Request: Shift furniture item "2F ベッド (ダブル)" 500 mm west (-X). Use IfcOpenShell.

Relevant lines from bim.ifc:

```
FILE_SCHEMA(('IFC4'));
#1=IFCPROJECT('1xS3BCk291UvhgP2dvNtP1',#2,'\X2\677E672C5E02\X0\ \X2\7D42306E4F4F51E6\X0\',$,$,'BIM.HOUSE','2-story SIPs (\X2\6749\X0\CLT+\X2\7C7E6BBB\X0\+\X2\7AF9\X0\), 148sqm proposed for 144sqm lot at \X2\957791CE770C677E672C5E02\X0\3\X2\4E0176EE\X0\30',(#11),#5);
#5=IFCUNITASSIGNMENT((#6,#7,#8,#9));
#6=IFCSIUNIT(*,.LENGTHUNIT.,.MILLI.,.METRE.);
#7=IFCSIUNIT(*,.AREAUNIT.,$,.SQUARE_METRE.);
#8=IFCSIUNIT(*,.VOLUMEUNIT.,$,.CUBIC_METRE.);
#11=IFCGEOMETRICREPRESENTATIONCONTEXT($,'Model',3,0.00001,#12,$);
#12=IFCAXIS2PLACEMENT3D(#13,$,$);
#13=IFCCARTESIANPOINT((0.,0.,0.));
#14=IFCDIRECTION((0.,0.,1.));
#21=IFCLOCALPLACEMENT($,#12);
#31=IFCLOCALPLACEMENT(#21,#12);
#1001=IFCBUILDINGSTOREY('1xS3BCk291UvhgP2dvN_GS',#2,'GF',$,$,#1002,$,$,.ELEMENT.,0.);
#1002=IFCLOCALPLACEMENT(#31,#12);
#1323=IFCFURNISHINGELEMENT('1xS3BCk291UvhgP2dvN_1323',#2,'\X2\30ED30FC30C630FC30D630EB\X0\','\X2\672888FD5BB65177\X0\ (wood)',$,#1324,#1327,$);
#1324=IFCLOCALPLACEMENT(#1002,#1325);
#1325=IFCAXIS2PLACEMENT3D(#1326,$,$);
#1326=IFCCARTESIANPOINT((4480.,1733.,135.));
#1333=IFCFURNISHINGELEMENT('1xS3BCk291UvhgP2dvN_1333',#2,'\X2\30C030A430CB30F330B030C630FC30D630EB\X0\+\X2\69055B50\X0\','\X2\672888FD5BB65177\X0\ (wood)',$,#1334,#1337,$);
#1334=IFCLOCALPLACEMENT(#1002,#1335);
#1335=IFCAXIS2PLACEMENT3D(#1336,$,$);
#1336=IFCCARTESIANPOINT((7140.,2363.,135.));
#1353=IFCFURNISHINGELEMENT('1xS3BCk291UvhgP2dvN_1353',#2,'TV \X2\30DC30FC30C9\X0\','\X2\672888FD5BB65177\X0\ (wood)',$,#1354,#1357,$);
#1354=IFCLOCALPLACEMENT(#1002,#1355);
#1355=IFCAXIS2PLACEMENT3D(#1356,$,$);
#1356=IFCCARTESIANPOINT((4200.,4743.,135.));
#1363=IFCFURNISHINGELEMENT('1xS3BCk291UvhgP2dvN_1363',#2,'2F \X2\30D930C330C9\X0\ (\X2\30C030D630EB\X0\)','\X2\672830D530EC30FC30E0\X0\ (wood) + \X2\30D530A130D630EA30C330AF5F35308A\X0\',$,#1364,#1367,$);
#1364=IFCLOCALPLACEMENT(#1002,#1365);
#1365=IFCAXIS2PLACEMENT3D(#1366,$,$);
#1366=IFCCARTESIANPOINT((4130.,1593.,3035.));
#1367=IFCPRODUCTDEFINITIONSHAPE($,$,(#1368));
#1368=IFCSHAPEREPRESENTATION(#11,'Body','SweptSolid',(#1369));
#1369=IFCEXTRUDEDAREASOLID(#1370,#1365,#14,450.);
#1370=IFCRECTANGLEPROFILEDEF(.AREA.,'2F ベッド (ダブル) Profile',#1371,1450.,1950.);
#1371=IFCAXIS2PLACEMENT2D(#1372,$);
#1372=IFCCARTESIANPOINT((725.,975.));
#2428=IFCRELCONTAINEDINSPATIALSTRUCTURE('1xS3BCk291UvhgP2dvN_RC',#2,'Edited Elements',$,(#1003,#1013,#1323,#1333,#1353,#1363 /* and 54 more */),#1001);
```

```python
import ifcopenshell
import ifcopenshell.api.geometry
import ifcopenshell.util.placement

model = ifcopenshell.open("bim.ifc")

item = model.by_guid("1xS3BCk291UvhgP2dvN_1363")
matrix = ifcopenshell.util.placement.get_local_placement(item.ObjectPlacement)
matrix[0, 3] -= 500.0
ifcopenshell.api.geometry.edit_object_placement(model, product=item, matrix=matrix, is_si=False)

print(ifcopenshell.util.placement.get_local_placement(item.ObjectPlacement).round(3) + 0.0)

model.write("bim_edited.ifc")
```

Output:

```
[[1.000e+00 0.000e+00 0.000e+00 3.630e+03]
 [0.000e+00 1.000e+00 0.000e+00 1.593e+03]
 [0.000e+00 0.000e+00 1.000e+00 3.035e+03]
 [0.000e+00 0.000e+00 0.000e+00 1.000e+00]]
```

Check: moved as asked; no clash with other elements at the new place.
